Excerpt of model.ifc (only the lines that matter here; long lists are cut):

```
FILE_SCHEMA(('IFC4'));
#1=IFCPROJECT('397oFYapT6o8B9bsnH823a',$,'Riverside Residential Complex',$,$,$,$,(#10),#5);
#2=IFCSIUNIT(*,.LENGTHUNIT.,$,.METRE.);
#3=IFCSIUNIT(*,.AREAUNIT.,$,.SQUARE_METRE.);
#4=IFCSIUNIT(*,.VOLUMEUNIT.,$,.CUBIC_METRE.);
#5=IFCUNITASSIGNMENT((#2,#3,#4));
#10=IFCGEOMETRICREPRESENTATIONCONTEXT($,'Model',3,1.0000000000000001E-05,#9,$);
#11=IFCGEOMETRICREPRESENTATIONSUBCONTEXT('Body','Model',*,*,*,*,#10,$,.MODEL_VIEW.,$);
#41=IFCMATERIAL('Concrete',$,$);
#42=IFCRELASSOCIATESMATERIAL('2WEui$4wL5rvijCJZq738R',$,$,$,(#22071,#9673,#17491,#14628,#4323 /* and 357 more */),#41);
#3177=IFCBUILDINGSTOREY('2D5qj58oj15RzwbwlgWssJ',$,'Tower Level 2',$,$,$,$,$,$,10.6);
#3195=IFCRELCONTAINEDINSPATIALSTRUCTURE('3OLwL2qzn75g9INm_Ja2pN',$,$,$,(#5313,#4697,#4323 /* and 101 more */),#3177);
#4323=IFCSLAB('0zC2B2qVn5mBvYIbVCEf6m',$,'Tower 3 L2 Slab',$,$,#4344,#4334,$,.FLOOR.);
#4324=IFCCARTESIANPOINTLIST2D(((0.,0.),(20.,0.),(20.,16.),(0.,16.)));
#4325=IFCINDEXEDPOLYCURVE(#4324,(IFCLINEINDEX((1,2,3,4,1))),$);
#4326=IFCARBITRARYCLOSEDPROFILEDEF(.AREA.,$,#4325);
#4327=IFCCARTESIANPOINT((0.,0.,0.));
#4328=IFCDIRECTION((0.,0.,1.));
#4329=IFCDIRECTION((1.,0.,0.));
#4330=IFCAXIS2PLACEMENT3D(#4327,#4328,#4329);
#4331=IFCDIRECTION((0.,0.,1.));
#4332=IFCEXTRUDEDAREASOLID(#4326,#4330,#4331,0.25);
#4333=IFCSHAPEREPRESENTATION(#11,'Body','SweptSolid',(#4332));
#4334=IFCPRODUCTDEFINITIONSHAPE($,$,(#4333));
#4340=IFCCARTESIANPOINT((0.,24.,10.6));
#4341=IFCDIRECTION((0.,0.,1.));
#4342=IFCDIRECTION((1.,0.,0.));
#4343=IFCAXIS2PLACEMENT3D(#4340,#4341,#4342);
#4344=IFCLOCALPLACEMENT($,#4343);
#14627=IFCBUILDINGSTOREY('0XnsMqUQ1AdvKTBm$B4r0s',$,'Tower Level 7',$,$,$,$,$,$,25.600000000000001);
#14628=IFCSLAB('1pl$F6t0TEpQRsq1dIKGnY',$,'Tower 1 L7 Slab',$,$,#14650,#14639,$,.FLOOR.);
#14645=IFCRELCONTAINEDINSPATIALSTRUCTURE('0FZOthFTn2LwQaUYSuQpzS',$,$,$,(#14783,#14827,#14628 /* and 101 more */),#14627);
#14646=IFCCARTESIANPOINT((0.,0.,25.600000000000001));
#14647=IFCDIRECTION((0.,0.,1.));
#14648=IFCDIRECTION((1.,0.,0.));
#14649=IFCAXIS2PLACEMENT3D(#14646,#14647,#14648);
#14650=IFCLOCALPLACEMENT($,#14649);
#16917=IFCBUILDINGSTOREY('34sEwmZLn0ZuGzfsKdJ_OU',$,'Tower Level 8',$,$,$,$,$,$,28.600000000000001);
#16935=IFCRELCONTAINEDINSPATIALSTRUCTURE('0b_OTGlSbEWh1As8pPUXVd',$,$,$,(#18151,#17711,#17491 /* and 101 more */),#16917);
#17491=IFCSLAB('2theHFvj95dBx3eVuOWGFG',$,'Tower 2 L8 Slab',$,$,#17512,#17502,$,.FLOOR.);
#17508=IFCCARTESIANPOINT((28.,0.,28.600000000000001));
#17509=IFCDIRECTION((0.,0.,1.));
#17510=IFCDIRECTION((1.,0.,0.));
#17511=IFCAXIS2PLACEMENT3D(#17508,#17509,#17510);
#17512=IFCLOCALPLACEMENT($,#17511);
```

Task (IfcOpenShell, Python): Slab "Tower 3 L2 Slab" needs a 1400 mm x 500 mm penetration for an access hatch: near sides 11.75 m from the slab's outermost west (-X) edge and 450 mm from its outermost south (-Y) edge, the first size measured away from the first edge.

```python
import numpy as np
import ifcopenshell
import ifcopenshell.api.feature
import ifcopenshell.api.geometry
import ifcopenshell.api.root
import ifcopenshell.geom
import ifcopenshell.util.placement
import ifcopenshell.util.representation
import ifcopenshell.util.shape
import ifcopenshell.util.unit

model = ifcopenshell.open("model.ifc")
unit_scale = ifcopenshell.util.unit.calculate_unit_scale(model)
settings = ifcopenshell.geom.settings()


def volume(element):
    """Net volume in cubic metres, openings subtracted."""
    shape = ifcopenshell.geom.create_shape(settings, element)
    return ifcopenshell.util.shape.get_volume(shape.geometry)


slab = model.by_id(4323)
before = volume(slab)

# Extent in the slab's own axes, in metres. The edges named are its -X and -Y sides.
slab_shape = ifcopenshell.geom.create_shape(settings, slab)
vertices = ifcopenshell.util.shape.get_vertices(slab_shape.geometry)
x_min, y_min, bottom = vertices.min(axis=0)
top = vertices[:, 2].max()

opening = ifcopenshell.api.root.create_entity(model, ifc_class="IfcOpeningElement", name="Access hatch opening", predefined_type="OPENING")
context = ifcopenshell.util.representation.get_context(model, "Model", "Body", "MODEL_VIEW")
width, depth = 1.4, 0.5
outline = [(0.0, 0.0), (width, 0.0), (width, depth), (0.0, depth), (0.0, 0.0)]
# Overshoot both faces by 50 mm so the cut is clean.
shape = ifcopenshell.api.geometry.add_slab_representation(
    model, context=context, depth=top - bottom + 0.1, polyline=outline
)
ifcopenshell.api.geometry.assign_representation(model, product=opening, representation=shape)

matrix = ifcopenshell.util.placement.get_local_placement(slab.ObjectPlacement)
matrix[:, 3] = matrix @ np.append(np.array([x_min + 11.75, y_min + 0.45, bottom - 0.05]) / unit_scale, 1.0)
ifcopenshell.api.geometry.edit_object_placement(model, product=opening, matrix=matrix, is_si=False)
ifcopenshell.api.feature.add_feature(model, feature=opening, element=slab)

after = volume(slab)

print(f"slab volume {before:.3f} -> {after:.3f} m3")

model.write("model_rev.ifc")
```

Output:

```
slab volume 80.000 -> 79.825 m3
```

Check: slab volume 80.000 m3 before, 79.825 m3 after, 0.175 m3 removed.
